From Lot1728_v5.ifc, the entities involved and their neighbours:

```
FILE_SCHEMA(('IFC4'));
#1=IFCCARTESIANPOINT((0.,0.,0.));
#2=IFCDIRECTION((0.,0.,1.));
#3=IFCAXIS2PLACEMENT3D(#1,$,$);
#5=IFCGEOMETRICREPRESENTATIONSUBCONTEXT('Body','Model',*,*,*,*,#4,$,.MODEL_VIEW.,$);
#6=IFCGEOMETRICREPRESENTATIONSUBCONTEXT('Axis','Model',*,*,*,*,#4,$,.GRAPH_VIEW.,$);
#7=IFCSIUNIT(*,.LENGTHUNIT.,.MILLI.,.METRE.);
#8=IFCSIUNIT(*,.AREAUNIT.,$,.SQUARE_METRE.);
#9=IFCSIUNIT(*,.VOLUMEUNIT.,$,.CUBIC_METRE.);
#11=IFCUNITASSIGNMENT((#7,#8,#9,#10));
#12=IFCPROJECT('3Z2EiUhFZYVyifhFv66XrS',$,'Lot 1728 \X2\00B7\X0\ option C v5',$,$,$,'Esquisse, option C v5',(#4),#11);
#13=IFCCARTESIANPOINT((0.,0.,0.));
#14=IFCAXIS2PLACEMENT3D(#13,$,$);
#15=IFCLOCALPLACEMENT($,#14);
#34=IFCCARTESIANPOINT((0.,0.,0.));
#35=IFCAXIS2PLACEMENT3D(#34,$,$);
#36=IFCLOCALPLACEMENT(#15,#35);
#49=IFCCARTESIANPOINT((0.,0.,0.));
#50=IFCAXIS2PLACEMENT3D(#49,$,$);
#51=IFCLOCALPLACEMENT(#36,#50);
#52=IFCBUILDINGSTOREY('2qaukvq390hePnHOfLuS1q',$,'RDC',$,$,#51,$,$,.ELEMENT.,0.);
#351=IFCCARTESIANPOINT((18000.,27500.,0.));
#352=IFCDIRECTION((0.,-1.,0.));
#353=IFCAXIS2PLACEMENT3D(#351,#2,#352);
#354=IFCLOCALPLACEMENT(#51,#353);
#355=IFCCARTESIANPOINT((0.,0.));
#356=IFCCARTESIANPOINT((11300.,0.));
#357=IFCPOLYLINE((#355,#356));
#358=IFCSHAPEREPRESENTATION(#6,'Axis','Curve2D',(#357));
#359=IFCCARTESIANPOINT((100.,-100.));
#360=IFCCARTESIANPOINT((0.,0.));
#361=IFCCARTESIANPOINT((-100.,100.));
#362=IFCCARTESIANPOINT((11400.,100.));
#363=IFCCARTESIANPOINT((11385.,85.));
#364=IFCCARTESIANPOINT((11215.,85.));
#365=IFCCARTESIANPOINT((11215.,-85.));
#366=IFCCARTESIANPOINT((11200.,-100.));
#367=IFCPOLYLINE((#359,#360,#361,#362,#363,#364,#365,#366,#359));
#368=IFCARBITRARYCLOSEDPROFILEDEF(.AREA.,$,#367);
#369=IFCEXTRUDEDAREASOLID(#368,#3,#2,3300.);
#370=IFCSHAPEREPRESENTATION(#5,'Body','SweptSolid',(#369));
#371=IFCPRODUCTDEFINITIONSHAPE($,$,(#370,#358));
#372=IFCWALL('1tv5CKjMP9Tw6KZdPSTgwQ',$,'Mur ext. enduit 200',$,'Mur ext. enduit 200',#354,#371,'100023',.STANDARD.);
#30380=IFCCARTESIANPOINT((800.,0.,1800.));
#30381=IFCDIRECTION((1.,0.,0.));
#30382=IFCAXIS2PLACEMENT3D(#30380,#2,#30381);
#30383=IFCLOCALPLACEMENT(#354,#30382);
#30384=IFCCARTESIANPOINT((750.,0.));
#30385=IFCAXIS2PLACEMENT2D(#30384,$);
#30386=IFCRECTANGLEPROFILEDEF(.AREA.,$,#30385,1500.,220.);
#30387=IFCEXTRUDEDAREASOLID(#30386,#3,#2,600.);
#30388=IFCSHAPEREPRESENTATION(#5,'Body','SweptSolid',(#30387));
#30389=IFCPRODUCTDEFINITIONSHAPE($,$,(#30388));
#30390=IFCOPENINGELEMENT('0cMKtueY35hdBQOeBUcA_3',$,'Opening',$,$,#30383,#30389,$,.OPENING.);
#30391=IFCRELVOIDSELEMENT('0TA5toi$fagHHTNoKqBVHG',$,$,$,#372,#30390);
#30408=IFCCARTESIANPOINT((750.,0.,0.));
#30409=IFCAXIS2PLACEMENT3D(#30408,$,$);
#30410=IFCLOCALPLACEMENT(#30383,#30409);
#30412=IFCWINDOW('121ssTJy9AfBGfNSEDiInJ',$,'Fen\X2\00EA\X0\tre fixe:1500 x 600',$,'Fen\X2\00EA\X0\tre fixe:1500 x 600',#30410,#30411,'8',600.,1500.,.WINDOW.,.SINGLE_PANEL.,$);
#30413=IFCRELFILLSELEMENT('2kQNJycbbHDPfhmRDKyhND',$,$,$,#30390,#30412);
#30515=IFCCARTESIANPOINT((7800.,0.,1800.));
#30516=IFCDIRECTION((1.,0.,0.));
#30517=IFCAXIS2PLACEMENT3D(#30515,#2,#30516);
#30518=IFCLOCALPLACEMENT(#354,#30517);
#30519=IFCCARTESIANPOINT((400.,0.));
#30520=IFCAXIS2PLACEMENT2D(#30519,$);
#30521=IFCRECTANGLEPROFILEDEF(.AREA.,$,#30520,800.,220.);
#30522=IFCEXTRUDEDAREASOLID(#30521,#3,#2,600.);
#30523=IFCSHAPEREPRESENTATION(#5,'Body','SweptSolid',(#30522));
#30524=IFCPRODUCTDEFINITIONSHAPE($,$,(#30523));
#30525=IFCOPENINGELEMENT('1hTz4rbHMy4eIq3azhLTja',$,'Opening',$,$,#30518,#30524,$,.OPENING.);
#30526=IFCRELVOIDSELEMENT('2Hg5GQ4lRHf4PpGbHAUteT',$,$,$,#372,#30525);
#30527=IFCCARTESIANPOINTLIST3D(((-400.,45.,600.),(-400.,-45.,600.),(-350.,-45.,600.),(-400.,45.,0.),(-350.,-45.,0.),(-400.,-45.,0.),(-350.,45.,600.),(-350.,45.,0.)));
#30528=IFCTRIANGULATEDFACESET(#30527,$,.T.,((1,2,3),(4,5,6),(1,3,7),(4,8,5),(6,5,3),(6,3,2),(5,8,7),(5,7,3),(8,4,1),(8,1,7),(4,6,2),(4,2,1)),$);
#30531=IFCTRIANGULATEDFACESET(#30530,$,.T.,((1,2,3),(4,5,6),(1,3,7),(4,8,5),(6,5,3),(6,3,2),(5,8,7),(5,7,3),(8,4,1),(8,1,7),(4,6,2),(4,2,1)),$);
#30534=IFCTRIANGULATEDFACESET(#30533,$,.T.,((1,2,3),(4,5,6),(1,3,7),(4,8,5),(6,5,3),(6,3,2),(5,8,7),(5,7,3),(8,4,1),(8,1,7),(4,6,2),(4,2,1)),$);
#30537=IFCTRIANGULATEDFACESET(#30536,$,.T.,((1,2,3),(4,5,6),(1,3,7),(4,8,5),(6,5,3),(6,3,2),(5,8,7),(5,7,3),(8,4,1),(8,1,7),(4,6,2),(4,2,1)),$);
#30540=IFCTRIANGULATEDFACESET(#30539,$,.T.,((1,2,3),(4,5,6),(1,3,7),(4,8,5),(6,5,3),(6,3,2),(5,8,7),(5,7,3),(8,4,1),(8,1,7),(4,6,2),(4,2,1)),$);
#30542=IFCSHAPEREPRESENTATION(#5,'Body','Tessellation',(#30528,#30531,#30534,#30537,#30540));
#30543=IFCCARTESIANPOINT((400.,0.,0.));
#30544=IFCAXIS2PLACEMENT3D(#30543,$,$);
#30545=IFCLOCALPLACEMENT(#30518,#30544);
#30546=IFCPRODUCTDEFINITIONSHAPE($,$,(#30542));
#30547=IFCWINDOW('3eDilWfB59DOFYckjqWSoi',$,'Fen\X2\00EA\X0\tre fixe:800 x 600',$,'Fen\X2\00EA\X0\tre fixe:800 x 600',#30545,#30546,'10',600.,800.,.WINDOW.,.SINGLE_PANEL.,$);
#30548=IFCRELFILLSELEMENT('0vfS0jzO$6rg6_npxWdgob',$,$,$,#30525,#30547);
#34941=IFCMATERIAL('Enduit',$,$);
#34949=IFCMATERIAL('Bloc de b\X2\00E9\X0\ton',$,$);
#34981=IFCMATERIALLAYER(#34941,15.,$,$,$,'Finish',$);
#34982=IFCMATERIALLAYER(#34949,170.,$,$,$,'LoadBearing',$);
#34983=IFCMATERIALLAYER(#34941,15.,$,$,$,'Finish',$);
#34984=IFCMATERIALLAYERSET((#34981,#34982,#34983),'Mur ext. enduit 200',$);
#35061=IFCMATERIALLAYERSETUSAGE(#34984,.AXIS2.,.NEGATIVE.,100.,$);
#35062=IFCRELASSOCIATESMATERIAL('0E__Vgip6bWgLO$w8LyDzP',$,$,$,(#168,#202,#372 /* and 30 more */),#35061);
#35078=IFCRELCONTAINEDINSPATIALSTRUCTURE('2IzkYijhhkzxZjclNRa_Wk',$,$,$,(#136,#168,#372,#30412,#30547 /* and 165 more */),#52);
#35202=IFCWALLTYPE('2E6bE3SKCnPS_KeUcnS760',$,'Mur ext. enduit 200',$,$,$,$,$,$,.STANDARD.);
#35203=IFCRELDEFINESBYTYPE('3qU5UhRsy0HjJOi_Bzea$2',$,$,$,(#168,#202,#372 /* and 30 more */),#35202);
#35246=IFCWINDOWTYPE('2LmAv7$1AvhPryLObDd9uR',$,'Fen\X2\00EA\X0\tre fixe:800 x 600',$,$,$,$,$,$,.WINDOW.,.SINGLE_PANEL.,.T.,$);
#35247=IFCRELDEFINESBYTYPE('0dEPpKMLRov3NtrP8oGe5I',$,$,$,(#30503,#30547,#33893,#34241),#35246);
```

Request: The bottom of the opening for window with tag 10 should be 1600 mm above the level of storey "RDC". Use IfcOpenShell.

```python
import numpy as np
import ifcopenshell
import ifcopenshell.api.geometry
import ifcopenshell.geom
import ifcopenshell.util.element
import ifcopenshell.util.placement
import ifcopenshell.util.shape
import ifcopenshell.util.unit

model = ifcopenshell.open("Lot1728_v5.ifc")
unit_scale = ifcopenshell.util.unit.calculate_unit_scale(model)

window = model.by_id(30547)
opening = window.FillsVoids[0].RelatingOpeningElement
storey = ifcopenshell.util.element.get_container(window, ifc_class="IfcBuildingStorey")
level = ifcopenshell.util.placement.get_local_placement(storey.ObjectPlacement)[2, 3]

# The opening's origin need not be at the sill, so measure its lowest point.
shape = ifcopenshell.geom.create_shape(ifcopenshell.geom.settings(), opening)
bottom = ifcopenshell.util.shape.get_shape_bottom_elevation(shape, shape.geometry) / unit_scale
dz = level + 1.6 / unit_scale - bottom

shift = np.array([0.0, 0.0, dz])
# The window is placed relative to its opening, so it follows when the opening moves.
matrix = ifcopenshell.util.placement.get_local_placement(opening.ObjectPlacement)
matrix[:3, 3] += shift
ifcopenshell.api.geometry.edit_object_placement(
    model, product=opening, matrix=matrix, is_si=False, should_transform_children=True
)

print(f"moved by {dz * unit_scale:+.3f} m")

model.write("Lot1728_v5_rev.ifc")
```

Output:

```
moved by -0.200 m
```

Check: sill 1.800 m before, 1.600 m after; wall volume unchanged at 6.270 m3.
